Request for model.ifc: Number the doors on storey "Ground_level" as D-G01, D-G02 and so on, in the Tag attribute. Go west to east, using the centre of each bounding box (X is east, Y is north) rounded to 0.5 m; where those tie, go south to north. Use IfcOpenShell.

First a look at what the model holds.

```python
import ifcopenshell
import ifcopenshell.util.element
import ifcopenshell.util.placement

model = ifcopenshell.open("model.ifc")
print(model.schema)
storey = next(s for s in model.by_type("IfcBuildingStorey") if s.Name == "Ground_level")
doors = [e for e in ifcopenshell.util.element.get_decomposition(storey) if e.is_a("IfcDoor")]
for e in sorted(doors, key=lambda e: e.id()):
    origin = ifcopenshell.util.placement.get_local_placement(e.ObjectPlacement)[:3, 3]
    print(e.id(), e.Tag, e.Name, origin.round(2) + 0.0, sep=" | ")
```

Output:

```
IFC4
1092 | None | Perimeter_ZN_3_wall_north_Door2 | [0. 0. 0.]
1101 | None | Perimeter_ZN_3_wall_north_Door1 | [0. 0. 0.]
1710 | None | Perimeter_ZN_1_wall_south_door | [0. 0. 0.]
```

```python
import ifcopenshell
import ifcopenshell.geom
import ifcopenshell.util.element
import ifcopenshell.util.shape

model = ifcopenshell.open("model.ifc")
settings = ifcopenshell.geom.settings()
settings.set("use-world-coords", True)


def centre(element):
    shape = ifcopenshell.geom.create_shape(settings, element)
    return ifcopenshell.util.shape.get_bbox_centroid(shape.geometry)


storey = next(s for s in model.by_type("IfcBuildingStorey") if s.Name == "Ground_level")
doors = [e for e in ifcopenshell.util.element.get_decomposition(storey) if e.is_a("IfcDoor")]

# Insertion points can sit at a corner or the storey origin, so sort by the geometry (in metres).
centres = {e: centre(e) for e in doors}
doors.sort(key=lambda e: (round(centres[e][0] / 0.5), centres[e][1]))

for i, e in enumerate(doors, start=1):
    number = f"D-G{i:02d}"
    e.Tag = number
    print(e.id(), number)

model.write("model-out.ifc")
```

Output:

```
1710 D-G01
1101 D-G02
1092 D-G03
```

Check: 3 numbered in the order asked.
